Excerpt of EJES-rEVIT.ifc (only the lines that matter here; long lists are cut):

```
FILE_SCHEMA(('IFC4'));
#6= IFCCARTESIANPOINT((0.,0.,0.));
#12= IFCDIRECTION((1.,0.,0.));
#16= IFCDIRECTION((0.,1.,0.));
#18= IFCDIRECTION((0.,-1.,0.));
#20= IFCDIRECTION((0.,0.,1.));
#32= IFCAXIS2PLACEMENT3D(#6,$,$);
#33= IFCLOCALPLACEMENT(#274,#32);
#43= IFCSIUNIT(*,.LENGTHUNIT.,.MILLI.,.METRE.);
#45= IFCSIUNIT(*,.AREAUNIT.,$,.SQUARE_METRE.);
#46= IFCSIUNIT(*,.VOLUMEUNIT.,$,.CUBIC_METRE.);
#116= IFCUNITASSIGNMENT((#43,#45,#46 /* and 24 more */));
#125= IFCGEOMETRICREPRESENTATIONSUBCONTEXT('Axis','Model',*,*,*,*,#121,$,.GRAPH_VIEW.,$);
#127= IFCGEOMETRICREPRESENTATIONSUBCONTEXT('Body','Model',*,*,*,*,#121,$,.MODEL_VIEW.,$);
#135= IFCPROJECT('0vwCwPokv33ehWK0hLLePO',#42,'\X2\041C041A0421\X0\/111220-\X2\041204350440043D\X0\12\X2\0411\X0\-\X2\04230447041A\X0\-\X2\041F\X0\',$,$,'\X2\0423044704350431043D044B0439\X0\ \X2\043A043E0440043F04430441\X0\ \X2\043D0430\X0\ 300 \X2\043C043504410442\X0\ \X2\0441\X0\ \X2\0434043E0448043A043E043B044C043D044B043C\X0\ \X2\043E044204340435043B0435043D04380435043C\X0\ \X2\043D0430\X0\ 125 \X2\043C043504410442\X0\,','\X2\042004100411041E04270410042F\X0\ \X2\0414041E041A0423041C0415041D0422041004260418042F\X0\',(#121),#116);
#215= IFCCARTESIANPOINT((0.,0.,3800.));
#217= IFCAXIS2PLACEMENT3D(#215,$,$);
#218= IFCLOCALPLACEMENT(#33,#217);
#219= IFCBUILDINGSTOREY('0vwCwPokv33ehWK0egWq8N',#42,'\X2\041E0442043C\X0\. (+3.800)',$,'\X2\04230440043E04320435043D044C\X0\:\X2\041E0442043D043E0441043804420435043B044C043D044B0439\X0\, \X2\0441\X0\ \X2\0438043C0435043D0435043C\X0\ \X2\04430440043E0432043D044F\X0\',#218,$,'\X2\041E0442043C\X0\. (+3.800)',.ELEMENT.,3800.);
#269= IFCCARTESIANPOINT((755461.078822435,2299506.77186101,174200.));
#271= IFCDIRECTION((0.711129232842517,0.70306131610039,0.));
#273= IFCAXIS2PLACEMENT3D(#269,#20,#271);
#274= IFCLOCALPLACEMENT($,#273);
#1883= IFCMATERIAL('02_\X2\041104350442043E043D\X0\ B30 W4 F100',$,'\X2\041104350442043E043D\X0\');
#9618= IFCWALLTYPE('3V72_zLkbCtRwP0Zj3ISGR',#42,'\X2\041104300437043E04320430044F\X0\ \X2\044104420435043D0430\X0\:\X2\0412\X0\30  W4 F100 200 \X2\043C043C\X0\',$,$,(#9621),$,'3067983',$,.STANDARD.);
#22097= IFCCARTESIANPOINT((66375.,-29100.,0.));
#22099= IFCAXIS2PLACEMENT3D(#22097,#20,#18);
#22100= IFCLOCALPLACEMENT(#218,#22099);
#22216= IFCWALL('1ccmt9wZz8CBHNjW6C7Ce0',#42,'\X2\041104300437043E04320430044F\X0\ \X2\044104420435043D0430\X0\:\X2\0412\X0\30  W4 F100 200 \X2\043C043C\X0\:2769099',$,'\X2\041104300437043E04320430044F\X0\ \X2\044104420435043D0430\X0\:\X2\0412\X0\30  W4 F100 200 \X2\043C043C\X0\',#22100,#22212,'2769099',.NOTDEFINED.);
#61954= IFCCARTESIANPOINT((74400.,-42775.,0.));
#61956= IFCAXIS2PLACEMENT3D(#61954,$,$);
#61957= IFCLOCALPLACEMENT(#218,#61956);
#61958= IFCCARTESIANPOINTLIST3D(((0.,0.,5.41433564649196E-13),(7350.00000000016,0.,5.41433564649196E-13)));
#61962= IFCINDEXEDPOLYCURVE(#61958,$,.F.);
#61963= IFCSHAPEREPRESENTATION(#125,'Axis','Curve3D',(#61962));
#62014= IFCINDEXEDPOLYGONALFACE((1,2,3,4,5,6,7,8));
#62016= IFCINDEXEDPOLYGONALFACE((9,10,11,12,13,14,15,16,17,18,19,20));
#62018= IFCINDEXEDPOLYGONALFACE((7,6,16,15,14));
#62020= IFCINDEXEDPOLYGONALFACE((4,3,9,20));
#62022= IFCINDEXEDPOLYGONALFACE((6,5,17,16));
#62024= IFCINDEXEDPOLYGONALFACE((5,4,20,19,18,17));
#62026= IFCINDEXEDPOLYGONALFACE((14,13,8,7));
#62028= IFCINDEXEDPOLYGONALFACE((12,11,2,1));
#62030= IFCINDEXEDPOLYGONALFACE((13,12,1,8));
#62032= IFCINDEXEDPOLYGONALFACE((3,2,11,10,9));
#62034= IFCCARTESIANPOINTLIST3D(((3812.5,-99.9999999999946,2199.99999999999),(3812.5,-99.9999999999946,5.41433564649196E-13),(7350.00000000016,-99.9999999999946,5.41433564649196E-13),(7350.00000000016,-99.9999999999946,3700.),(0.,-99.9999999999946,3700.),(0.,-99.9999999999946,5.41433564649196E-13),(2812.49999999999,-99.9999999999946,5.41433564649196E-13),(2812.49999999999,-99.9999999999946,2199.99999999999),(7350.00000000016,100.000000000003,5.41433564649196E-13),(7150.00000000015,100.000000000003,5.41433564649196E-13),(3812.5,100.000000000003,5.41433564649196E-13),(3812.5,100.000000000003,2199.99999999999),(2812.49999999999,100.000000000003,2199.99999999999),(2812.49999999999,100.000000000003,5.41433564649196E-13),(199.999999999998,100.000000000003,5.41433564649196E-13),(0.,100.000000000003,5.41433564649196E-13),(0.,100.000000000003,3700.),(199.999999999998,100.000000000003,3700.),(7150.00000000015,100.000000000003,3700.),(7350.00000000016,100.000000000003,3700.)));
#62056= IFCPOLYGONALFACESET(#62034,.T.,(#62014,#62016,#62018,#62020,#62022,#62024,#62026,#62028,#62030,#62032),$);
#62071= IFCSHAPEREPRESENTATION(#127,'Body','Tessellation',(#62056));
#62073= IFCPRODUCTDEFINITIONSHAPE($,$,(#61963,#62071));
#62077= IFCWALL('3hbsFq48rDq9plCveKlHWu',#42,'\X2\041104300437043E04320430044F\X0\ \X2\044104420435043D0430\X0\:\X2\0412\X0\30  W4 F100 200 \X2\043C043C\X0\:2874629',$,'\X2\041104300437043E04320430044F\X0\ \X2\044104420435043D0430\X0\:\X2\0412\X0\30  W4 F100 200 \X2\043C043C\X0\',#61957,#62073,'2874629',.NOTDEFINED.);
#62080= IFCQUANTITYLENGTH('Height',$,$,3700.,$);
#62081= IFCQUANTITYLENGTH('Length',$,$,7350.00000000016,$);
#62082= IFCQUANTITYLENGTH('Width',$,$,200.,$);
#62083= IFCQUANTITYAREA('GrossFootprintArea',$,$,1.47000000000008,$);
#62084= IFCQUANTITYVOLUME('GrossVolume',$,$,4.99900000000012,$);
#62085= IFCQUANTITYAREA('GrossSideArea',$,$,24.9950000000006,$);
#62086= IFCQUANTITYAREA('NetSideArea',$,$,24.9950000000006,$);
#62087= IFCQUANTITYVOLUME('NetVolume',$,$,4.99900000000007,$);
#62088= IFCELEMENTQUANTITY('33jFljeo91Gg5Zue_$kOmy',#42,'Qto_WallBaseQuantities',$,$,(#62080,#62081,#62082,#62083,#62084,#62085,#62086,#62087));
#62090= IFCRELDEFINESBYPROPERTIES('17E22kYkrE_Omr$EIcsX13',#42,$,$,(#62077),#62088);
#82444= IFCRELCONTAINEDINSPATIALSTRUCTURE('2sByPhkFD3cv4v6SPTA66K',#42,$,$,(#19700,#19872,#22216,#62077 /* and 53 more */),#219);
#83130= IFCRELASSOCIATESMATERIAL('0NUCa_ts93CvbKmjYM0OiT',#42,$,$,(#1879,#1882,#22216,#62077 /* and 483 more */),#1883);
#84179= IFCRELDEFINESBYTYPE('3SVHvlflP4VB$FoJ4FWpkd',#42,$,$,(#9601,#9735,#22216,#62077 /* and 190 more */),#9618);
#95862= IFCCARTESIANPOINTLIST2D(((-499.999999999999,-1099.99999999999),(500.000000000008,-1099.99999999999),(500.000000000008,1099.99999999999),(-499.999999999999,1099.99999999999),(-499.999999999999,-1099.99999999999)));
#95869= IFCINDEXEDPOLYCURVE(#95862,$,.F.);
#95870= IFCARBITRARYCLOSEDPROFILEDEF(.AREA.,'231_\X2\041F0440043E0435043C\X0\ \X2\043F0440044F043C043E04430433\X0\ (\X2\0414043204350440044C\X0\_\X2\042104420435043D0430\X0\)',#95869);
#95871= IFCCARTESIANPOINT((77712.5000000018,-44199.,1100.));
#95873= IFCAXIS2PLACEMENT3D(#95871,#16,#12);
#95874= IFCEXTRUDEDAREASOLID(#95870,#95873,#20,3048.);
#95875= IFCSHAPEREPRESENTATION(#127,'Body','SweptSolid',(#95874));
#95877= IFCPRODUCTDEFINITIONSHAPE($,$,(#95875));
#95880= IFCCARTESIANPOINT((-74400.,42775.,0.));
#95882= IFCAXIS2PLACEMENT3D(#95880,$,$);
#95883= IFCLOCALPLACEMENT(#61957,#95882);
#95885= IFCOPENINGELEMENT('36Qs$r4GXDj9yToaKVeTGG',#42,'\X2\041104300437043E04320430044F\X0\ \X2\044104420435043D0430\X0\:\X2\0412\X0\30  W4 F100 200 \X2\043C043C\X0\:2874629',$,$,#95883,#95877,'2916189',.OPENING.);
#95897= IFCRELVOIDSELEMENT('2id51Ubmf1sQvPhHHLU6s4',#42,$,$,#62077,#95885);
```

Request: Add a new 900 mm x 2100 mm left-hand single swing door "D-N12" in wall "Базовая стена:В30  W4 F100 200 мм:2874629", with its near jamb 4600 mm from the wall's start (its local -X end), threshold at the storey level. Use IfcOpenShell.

```python
import numpy as np
import ifcopenshell
import ifcopenshell.api.feature
import ifcopenshell.api.geometry
import ifcopenshell.api.pset
import ifcopenshell.api.root
import ifcopenshell.api.spatial
import ifcopenshell.geom
import ifcopenshell.util.element
import ifcopenshell.util.placement
import ifcopenshell.util.representation
import ifcopenshell.util.shape
import ifcopenshell.util.unit

model = ifcopenshell.open("EJES-rEVIT.ifc")
unit_scale = ifcopenshell.util.unit.calculate_unit_scale(model)
area_scale = ifcopenshell.util.unit.calculate_unit_scale(model, "AREAUNIT")
volume_scale = ifcopenshell.util.unit.calculate_unit_scale(model, "VOLUMEUNIT")
settings = ifcopenshell.geom.settings()


def volume(element):
    """Net volume in cubic metres, openings subtracted."""
    shape = ifcopenshell.geom.create_shape(settings, element)
    return ifcopenshell.util.shape.get_volume(shape.geometry)


wall = model.by_guid("3hbsFq48rDq9plCveKlHWu")
storey = ifcopenshell.util.element.get_container(wall, ifc_class="IfcBuildingStorey")
context = ifcopenshell.util.representation.get_context(model, "Model", "Body", "MODEL_VIEW")
before = volume(wall)

width, height, from_end, sill = 0.9, 2.1, 4.6, 0.0  # metres

# The wall runs along its own X axis, and the end named is its -X end.
wall_shape = ifcopenshell.geom.create_shape(settings, wall)
x, y, z = ifcopenshell.util.shape.get_vertices(wall_shape.geometry).T
start = x.min() + from_end
face, thickness = float(y.min()), float(y.max() - y.min())
wall_matrix = ifcopenshell.util.placement.get_local_placement(wall.ObjectPlacement)
level = ifcopenshell.util.placement.get_local_placement(storey.ObjectPlacement)[2, 3]


def in_wall(x, y):
    """Placement at x, y metres in the wall's axes, at sill height."""
    matrix = wall_matrix.copy()
    matrix[:, 3] = wall_matrix @ np.array([x / unit_scale, y / unit_scale, 0.0, 1.0])
    matrix[2, 3] = level + sill / unit_scale
    return matrix


# Opening: a box that overshoots both wall faces by 50 mm.
opening = ifcopenshell.api.root.create_entity(model, ifc_class="IfcOpeningElement", predefined_type="OPENING")
box = ifcopenshell.api.geometry.add_wall_representation(
    model, context=context, length=width, height=height, thickness=thickness + 0.1
)
ifcopenshell.api.geometry.assign_representation(model, product=opening, representation=box)
ifcopenshell.api.geometry.edit_object_placement(model, product=opening, matrix=in_wall(start, face - 0.05), is_si=False)
ifcopenshell.api.feature.add_feature(model, feature=opening, element=wall)

door = ifcopenshell.api.root.create_entity(model, ifc_class="IfcDoor", name="D-N12", predefined_type="DOOR")
door.OverallWidth, door.OverallHeight = width / unit_scale, height / unit_scale
door.OperationType = "SINGLE_SWING_LEFT"
body = ifcopenshell.api.geometry.add_door_representation(
    model,
    context=context,
    overall_width=door.OverallWidth,
    overall_height=door.OverallHeight,
    operation_type="SINGLE_SWING_LEFT",
    lining_properties={"LiningDepth": thickness / unit_scale, "ThresholdDepth": thickness / unit_scale},
)
ifcopenshell.api.geometry.assign_representation(model, product=door, representation=body)
ifcopenshell.api.spatial.assign_container(model, products=[door], relating_structure=storey)
ifcopenshell.api.feature.add_filling(model, opening=opening, element=door)

# The lining spans the wall, so the door starts at the wall face.
ifcopenshell.api.geometry.edit_object_placement(model, product=door, matrix=in_wall(start, face), is_si=False)

after = volume(wall)

# Update the wall's stored quantities.
qto = model.by_id(ifcopenshell.util.element.get_pset(wall, "Qto_WallBaseQuantities", should_inherit=False)["id"])
ifcopenshell.api.pset.edit_qto(model, qto=qto, properties={
    "NetSideArea": after / thickness / area_scale,
    "NetVolume": after / volume_scale,
})

print(f"wall volume {before:.3f} -> {after:.3f} m3")

model.write("EJES-rEVIT_v2.ifc")
```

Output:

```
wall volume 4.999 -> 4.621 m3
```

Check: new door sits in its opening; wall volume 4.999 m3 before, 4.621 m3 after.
